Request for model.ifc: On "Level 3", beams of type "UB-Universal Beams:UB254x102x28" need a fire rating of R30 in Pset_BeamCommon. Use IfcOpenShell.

First a look at what the model holds.

```python
import ifcopenshell
import ifcopenshell.util.element

model = ifcopenshell.open("model.ifc")
print(model.schema)
storey = next(s for s in model.by_type("IfcBuildingStorey") if s.Name == "Level 3")
beams = [e for e in ifcopenshell.util.element.get_decomposition(storey) if e.is_a("IfcBeam")]
seen = {}
for e in beams:
    element_type = ifcopenshell.util.element.get_type(e)
    key = (element_type.Name if element_type != e and element_type else None, ifcopenshell.util.element.get_pset(e, "Pset_BeamCommon", "FireRating"))
    seen[key] = seen.get(key, 0) + 1
for (name, value), count in sorted(seen.items(), key=str):
    print(count, "x", name, "|", value)
```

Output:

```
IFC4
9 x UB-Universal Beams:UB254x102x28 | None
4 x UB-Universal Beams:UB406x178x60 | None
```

```python
import ifcopenshell
import ifcopenshell.api.pset
import ifcopenshell.util.element

model = ifcopenshell.open("model.ifc")

storey = next(s for s in model.by_type("IfcBuildingStorey") if s.Name == "Level 3")
beams = [e for e in ifcopenshell.util.element.get_decomposition(storey) if e.is_a("IfcBeam")]

count = 0
for e in beams:
    element_type = ifcopenshell.util.element.get_type(e)
    if element_type in (None, e) or element_type.Name != "UB-Universal Beams:UB254x102x28":
        continue
    # add_pset returns the element's existing set when there is one.
    pset = ifcopenshell.api.pset.add_pset(model, product=e, name="Pset_BeamCommon")
    ifcopenshell.api.pset.edit_pset(model, pset=pset, properties={"FireRating": "R30"})
    count += 1

print(count, "beams updated")

model.write("model_rev.ifc")
```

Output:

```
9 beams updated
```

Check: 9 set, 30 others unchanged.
